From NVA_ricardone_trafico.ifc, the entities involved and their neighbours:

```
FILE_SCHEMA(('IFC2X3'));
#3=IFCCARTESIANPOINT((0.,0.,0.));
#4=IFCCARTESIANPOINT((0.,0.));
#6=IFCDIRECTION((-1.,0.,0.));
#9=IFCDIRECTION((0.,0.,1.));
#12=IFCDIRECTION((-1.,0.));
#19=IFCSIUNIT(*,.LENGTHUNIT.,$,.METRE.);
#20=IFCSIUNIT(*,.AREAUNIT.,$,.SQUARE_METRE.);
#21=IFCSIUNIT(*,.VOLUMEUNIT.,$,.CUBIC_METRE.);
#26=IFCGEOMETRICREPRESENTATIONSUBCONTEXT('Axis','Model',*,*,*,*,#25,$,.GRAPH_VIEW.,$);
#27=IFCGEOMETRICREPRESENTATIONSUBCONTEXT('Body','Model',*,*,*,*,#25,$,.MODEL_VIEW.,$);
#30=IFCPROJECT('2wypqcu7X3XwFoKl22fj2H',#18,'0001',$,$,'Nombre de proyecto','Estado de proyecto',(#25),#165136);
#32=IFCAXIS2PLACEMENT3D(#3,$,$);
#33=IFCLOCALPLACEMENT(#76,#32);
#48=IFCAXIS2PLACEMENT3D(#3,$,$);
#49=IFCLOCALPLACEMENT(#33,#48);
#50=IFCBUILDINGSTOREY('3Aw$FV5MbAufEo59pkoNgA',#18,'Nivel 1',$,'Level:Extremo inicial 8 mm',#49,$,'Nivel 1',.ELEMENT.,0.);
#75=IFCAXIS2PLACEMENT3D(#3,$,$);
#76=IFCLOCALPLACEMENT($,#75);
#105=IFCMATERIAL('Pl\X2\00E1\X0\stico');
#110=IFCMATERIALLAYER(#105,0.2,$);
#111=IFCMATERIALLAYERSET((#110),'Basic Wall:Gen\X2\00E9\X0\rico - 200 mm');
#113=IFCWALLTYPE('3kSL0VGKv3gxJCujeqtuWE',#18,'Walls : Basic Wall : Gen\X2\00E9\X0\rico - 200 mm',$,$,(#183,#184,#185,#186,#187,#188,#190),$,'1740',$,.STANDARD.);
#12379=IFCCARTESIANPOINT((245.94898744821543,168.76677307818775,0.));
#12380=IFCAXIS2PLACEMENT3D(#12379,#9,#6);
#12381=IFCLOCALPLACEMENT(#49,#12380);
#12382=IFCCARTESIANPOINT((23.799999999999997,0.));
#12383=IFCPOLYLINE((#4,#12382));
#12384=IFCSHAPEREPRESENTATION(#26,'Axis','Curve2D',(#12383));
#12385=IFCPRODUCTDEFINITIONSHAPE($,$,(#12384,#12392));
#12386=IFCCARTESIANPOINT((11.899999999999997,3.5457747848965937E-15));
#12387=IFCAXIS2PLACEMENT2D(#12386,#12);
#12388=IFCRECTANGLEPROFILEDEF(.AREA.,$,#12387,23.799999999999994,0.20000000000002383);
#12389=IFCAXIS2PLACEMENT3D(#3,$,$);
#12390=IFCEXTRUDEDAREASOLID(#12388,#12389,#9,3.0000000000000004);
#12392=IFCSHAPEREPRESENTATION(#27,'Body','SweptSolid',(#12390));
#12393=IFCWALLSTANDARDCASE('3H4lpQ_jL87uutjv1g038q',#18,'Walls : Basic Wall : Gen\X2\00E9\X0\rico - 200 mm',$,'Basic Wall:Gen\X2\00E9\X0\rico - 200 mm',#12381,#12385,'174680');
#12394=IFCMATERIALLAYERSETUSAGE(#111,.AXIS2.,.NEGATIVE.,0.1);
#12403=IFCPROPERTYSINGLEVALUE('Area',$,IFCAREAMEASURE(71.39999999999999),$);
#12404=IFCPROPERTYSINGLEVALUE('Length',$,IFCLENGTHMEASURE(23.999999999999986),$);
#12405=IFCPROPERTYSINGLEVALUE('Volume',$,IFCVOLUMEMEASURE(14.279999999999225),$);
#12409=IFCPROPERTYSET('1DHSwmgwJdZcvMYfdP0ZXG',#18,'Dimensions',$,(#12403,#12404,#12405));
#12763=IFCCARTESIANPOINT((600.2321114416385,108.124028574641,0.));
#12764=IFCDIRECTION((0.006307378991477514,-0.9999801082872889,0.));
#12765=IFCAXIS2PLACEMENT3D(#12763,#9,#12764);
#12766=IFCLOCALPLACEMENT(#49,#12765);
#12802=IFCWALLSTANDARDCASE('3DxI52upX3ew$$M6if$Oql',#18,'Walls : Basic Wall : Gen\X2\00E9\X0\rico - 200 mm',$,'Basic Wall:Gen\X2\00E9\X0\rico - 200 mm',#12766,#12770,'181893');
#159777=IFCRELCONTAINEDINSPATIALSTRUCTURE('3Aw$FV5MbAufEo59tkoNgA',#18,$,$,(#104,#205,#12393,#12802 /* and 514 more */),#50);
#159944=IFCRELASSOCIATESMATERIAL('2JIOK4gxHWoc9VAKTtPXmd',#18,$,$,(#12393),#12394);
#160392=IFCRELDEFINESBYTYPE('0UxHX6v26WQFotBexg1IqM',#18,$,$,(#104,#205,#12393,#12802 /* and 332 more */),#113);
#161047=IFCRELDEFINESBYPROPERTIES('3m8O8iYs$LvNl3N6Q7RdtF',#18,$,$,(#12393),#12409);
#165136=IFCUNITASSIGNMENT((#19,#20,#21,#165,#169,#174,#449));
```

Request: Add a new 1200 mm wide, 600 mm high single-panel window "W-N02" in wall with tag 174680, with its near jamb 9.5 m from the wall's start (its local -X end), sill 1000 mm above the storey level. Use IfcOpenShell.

```python
import numpy as np
import ifcopenshell
import ifcopenshell.api.feature
import ifcopenshell.api.geometry
import ifcopenshell.api.pset
import ifcopenshell.api.root
import ifcopenshell.api.spatial
import ifcopenshell.api.type
import ifcopenshell.geom
import ifcopenshell.util.element
import ifcopenshell.util.placement
import ifcopenshell.util.representation
import ifcopenshell.util.shape
import ifcopenshell.util.unit

model = ifcopenshell.open("NVA_ricardone_trafico.ifc")
unit_scale = ifcopenshell.util.unit.calculate_unit_scale(model)
area_scale = ifcopenshell.util.unit.calculate_unit_scale(model, "AREAUNIT")
volume_scale = ifcopenshell.util.unit.calculate_unit_scale(model, "VOLUMEUNIT")
settings = ifcopenshell.geom.settings()


def volume(element):
    """Net volume in cubic metres, openings subtracted."""
    shape = ifcopenshell.geom.create_shape(settings, element)
    return ifcopenshell.util.shape.get_volume(shape.geometry)


wall = model.by_id(12393)
storey = ifcopenshell.util.element.get_container(wall, ifc_class="IfcBuildingStorey")
context = ifcopenshell.util.representation.get_context(model, "Model", "Body", "MODEL_VIEW")
before = volume(wall)

width, height, from_end, sill = 1.2, 0.6, 9.5, 1  # metres

# The wall runs along its own X axis, and the end named is its -X end.
wall_shape = ifcopenshell.geom.create_shape(settings, wall)
x, y, z = ifcopenshell.util.shape.get_vertices(wall_shape.geometry).T
start = x.min() + from_end
face, thickness = float(y.min()), float(y.max() - y.min())
wall_matrix = ifcopenshell.util.placement.get_local_placement(wall.ObjectPlacement)
level = ifcopenshell.util.placement.get_local_placement(storey.ObjectPlacement)[2, 3]


def in_wall(x, y):
    """Placement at x, y metres in the wall's axes, at sill height."""
    matrix = wall_matrix.copy()
    matrix[:, 3] = wall_matrix @ np.array([x / unit_scale, y / unit_scale, 0.0, 1.0])
    matrix[2, 3] = level + sill / unit_scale
    return matrix


# Opening: a box that overshoots both wall faces by 50 mm.
opening = ifcopenshell.api.root.create_entity(model, ifc_class="IfcOpeningElement")
box = ifcopenshell.api.geometry.add_wall_representation(
    model, context=context, length=width, height=height, thickness=thickness + 0.1
)
ifcopenshell.api.geometry.assign_representation(model, product=opening, representation=box)
ifcopenshell.api.geometry.edit_object_placement(model, product=opening, matrix=in_wall(start, face - 0.05), is_si=False)
ifcopenshell.api.feature.add_feature(model, feature=opening, element=wall)

window = ifcopenshell.api.root.create_entity(model, ifc_class="IfcWindow", name="W-N02")
window.OverallWidth, window.OverallHeight = width / unit_scale, height / unit_scale
body = ifcopenshell.api.geometry.add_window_representation(
    model,
    context=context,
    overall_width=window.OverallWidth,
    overall_height=window.OverallHeight,
    partition_type="SINGLE_PANEL",
)
ifcopenshell.api.geometry.assign_representation(model, product=window, representation=body)
ifcopenshell.api.spatial.assign_container(model, products=[window], relating_structure=storey)
fills = ifcopenshell.api.feature.add_filling(model, opening=opening, element=window)
fills.OwnerHistory = window.OwnerHistory  # required in IFC2X3

# IFC2X3 keeps the operation on the window style.
style = ifcopenshell.api.root.create_entity(model, ifc_class="IfcWindowStyle", name="W-N02")
style.OperationType, style.ConstructionType = "SINGLE_PANEL", "NOTDEFINED"
style.ParameterTakesPrecedence = style.Sizeable = False
ifcopenshell.api.type.assign_type(model, related_objects=[window], relating_type=style)

# Centre the window in the wall's thickness.
ifcopenshell.api.geometry.edit_object_placement(model, product=window, matrix=in_wall(start, face), is_si=False)
window_shape = ifcopenshell.geom.create_shape(settings, window)
depth = ifcopenshell.util.shape.get_vertices(window_shape.geometry)[:, 1]
offset = face + thickness / 2 - (depth.min() + depth.max()) / 2
ifcopenshell.api.geometry.edit_object_placement(model, product=window, matrix=in_wall(start, offset), is_si=False)

after = volume(wall)

# Update the wall's stored quantities.
pset = model.by_id(ifcopenshell.util.element.get_pset(wall, "Dimensions", should_inherit=False)["id"])
ifcopenshell.api.pset.edit_pset(model, pset=pset, properties={
    "Area": model.create_entity("IfcAreaMeasure", after / thickness / area_scale),
    "Volume": model.create_entity("IfcVolumeMeasure", after / volume_scale),
})

print(f"wall volume {before:.3f} -> {after:.3f} m3")

model.write("NVA_ricardone_trafico_rev.ifc")
```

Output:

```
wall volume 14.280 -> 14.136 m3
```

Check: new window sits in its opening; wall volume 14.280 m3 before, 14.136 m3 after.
